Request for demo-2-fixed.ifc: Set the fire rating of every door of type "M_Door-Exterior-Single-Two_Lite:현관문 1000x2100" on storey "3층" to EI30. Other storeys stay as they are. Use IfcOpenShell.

First a look at what the model holds.

```python
import ifcopenshell
import ifcopenshell.util.element

model = ifcopenshell.open("demo-2-fixed.ifc")
print(model.schema)
storey = next(s for s in model.by_type("IfcBuildingStorey") if s.Name == "3층")
doors = [e for e in ifcopenshell.util.element.get_decomposition(storey) if e.is_a("IfcDoor")]
seen = {}
for e in doors:
    element_type = ifcopenshell.util.element.get_type(e)
    key = (element_type.Name if element_type != e and element_type else None, ifcopenshell.util.element.get_pset(e, "Pset_DoorCommon", "FireRating"))
    seen[key] = seen.get(key, 0) + 1
for (name, value), count in sorted(seen.items(), key=str):
    print(count, "x", name, "|", value)
```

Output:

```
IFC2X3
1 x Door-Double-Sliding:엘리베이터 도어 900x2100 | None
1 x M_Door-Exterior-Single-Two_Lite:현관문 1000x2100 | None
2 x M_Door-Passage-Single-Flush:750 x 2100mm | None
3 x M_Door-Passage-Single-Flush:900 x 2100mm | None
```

```python
import ifcopenshell
import ifcopenshell.api.pset
import ifcopenshell.util.element

model = ifcopenshell.open("demo-2-fixed.ifc")

storey = next(s for s in model.by_type("IfcBuildingStorey") if s.Name == "3층")
doors = [e for e in ifcopenshell.util.element.get_decomposition(storey) if e.is_a("IfcDoor")]

count = 0
for e in doors:
    element_type = ifcopenshell.util.element.get_type(e)
    if element_type in (None, e) or element_type.Name != "M_Door-Exterior-Single-Two_Lite:현관문 1000x2100":
        continue
    # add_pset returns the element's existing set when there is one.
    pset = ifcopenshell.api.pset.add_pset(model, product=e, name="Pset_DoorCommon")
    ifcopenshell.api.pset.edit_pset(model, pset=pset, properties={"FireRating": "EI30"})
    count += 1

print(count, "doors updated")

model.write("demo-2-fixed_updated.ifc")
```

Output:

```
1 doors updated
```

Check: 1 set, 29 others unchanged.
